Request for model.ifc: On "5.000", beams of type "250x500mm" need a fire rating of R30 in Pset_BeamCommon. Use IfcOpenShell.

First a look at what the model holds.

```python
import ifcopenshell
import ifcopenshell.util.element

model = ifcopenshell.open("model.ifc")
print(model.schema)
storey = next(s for s in model.by_type("IfcBuildingStorey") if s.Name == "5.000")
beams = [e for e in ifcopenshell.util.element.get_decomposition(storey) if e.is_a("IfcBeam")]
seen = {}
for e in beams:
    element_type = ifcopenshell.util.element.get_type(e)
    key = (element_type.Name if element_type != e and element_type else None, ifcopenshell.util.element.get_pset(e, "Pset_BeamCommon", "FireRating"))
    seen[key] = seen.get(key, 0) + 1
for (name, value), count in sorted(seen.items(), key=str):
    print(count, "x", name, "|", value)
```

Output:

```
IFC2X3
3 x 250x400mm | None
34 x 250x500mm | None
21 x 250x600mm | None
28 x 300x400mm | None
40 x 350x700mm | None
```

```python
import ifcopenshell
import ifcopenshell.api.pset
import ifcopenshell.util.element

model = ifcopenshell.open("model.ifc")

storey = next(s for s in model.by_type("IfcBuildingStorey") if s.Name == "5.000")
beams = [e for e in ifcopenshell.util.element.get_decomposition(storey) if e.is_a("IfcBeam")]

count = 0
for e in beams:
    element_type = ifcopenshell.util.element.get_type(e)
    if element_type in (None, e) or element_type.Name != "250x500mm":
        continue
    # add_pset returns the element's existing set when there is one.
    pset = ifcopenshell.api.pset.add_pset(model, product=e, name="Pset_BeamCommon")
    ifcopenshell.api.pset.edit_pset(model, pset=pset, properties={"FireRating": "R30"})
    count += 1

print(count, "beams updated")

model.write("model_rev.ifc")
```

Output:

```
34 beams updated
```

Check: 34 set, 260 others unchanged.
